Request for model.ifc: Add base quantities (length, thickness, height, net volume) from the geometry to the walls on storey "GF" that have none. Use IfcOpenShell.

First a look at what the model holds.

```python
import ifcopenshell
import ifcopenshell.util.element
import ifcopenshell.util.unit

model = ifcopenshell.open("model.ifc")
print(model.schema)
for unit_type in ("LENGTHUNIT", "AREAUNIT", "VOLUMEUNIT"):
    print(unit_type, ifcopenshell.util.unit.calculate_unit_scale(model, unit_type))
storey = next(s for s in model.by_type("IfcBuildingStorey") if s.Name == "GF")
walls = [e for e in ifcopenshell.util.element.get_decomposition(storey) if e.is_a("IfcWall")]
for e in sorted(walls, key=lambda e: e.id()):
    print(e.id(), e.is_a(), e.Name, list(ifcopenshell.util.element.get_psets(e, qtos_only=True)), sep=" | ")
```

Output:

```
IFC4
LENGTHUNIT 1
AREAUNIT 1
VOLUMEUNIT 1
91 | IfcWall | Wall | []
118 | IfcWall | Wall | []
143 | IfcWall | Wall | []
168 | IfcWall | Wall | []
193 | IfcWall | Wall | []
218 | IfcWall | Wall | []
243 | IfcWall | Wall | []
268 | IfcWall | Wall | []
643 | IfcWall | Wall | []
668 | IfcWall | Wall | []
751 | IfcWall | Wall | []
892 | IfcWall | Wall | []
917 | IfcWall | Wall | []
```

```python
import ifcopenshell
import ifcopenshell.api.pset
import ifcopenshell.geom
import ifcopenshell.util.element
import ifcopenshell.util.shape
import ifcopenshell.util.unit

model = ifcopenshell.open("model.ifc")
unit_scale = ifcopenshell.util.unit.calculate_unit_scale(model)
volume_scale = ifcopenshell.util.unit.calculate_unit_scale(model, "VOLUMEUNIT")
settings = ifcopenshell.geom.settings()

storey = next(s for s in model.by_type("IfcBuildingStorey") if s.Name == "GF")
walls = [e for e in ifcopenshell.util.element.get_decomposition(storey) if e.is_a("IfcWall")]

for e in sorted(walls, key=lambda e: e.id()):
    if ifcopenshell.util.element.get_psets(e, qtos_only=True, should_inherit=False):
        continue
    # Geometry comes back in metres, in the element's own axes.
    shape = ifcopenshell.geom.create_shape(settings, e)
    values = {
        "Length": ifcopenshell.util.shape.get_x(shape.geometry) / unit_scale,
        "Width": ifcopenshell.util.shape.get_y(shape.geometry) / unit_scale,
        "Height": ifcopenshell.util.shape.get_z(shape.geometry) / unit_scale,
        "NetVolume": ifcopenshell.util.shape.get_volume(shape.geometry) / volume_scale,
    }
    qto = ifcopenshell.api.pset.add_qto(model, product=e, name="Qto_WallBaseQuantities")
    ifcopenshell.api.pset.edit_qto(model, qto=qto, properties=values)
    print(e.id(), {k: round(v, 3) for k, v in values.items()})

model.write("model-out.ifc")
```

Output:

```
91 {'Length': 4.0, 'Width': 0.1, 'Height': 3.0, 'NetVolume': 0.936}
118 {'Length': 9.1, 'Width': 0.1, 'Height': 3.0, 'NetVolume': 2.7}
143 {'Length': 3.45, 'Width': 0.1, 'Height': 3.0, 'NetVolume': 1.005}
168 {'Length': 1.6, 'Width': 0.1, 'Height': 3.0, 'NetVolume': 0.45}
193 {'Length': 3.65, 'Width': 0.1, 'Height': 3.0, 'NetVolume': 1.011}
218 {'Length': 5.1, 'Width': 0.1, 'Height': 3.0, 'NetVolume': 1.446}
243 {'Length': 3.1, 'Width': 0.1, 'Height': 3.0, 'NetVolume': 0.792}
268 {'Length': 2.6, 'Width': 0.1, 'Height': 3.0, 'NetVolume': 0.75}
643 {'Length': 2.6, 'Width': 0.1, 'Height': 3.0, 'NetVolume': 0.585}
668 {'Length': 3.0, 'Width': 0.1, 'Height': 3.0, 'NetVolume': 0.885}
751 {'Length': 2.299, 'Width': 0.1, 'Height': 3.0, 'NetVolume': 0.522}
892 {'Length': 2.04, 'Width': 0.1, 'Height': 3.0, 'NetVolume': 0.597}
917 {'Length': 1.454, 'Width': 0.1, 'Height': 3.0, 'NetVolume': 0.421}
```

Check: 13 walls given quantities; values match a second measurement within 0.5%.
